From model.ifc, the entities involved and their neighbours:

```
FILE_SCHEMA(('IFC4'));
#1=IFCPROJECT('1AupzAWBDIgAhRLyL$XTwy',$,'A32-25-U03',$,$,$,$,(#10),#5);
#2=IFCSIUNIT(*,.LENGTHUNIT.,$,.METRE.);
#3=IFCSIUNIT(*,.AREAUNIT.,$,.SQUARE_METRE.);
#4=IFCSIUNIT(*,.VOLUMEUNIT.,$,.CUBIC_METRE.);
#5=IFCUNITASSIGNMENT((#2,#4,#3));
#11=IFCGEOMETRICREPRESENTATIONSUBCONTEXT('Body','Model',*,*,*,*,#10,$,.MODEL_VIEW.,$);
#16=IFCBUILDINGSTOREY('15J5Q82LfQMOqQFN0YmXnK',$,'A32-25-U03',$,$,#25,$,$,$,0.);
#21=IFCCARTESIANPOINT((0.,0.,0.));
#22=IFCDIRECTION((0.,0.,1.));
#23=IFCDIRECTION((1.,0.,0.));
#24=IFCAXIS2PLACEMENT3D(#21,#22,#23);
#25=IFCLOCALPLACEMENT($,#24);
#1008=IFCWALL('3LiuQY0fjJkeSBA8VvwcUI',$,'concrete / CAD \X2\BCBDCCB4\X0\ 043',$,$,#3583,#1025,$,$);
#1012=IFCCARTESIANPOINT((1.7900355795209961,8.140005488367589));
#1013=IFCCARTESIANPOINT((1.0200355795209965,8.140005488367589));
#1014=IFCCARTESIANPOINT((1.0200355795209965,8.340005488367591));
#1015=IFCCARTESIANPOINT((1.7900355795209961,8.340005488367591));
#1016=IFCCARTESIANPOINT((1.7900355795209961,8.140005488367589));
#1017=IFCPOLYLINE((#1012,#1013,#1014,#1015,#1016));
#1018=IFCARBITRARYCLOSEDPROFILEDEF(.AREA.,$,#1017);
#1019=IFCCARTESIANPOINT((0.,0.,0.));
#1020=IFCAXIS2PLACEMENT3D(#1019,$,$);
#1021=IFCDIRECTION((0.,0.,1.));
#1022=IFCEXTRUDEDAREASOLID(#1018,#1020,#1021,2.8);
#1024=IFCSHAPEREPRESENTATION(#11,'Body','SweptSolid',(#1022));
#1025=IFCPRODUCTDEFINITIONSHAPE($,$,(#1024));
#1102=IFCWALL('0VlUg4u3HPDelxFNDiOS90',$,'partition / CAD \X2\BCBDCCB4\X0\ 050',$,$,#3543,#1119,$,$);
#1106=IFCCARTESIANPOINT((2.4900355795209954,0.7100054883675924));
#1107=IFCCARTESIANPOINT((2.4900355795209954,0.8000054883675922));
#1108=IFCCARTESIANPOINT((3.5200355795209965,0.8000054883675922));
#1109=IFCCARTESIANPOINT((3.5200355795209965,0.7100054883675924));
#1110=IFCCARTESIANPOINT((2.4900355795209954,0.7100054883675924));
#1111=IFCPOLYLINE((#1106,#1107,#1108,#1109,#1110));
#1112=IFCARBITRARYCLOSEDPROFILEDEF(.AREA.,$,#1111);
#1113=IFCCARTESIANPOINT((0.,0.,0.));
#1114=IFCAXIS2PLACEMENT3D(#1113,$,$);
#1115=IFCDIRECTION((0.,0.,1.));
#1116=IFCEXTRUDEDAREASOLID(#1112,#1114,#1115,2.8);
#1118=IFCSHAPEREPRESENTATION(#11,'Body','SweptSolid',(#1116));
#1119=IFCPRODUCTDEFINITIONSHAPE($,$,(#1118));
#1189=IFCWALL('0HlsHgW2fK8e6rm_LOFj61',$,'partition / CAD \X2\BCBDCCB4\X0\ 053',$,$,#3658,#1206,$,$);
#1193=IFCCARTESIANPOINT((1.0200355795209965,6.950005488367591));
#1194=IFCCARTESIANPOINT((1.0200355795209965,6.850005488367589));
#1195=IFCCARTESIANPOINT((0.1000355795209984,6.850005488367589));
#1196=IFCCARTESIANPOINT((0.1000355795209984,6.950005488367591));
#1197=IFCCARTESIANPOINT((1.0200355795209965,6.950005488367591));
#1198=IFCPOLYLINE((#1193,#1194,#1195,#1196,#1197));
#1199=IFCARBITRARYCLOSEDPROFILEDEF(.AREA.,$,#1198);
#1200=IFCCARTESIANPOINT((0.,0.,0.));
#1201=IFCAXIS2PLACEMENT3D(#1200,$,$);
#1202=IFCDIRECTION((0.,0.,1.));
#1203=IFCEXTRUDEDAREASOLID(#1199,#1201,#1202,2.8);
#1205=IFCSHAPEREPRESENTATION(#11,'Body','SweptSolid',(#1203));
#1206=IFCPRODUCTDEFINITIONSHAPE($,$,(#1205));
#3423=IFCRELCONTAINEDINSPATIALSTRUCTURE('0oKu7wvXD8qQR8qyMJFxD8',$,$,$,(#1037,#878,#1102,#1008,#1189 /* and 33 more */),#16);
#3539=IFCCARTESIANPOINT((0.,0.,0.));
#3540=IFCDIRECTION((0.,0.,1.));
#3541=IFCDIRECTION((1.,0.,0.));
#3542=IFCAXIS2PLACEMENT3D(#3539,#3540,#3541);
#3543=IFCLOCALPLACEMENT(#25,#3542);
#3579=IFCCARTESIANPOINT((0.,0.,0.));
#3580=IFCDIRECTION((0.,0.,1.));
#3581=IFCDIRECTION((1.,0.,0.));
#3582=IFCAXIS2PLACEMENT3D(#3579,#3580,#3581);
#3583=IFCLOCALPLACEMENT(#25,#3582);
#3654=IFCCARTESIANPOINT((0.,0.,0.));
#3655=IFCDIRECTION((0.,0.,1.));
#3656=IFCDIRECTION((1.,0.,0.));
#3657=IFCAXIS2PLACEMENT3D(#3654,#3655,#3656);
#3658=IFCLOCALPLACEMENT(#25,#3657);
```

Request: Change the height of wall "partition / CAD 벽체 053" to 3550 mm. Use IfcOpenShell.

```python
import ifcopenshell
import ifcopenshell.geom
import ifcopenshell.util.representation
import ifcopenshell.util.shape

model = ifcopenshell.open("model.ifc")
settings = ifcopenshell.geom.settings()


def volume(element):
    """Net volume in cubic metres, openings subtracted."""
    shape = ifcopenshell.geom.create_shape(settings, element)
    return ifcopenshell.util.shape.get_volume(shape.geometry)


wall = model.by_id(1189)
before = volume(wall)

body = ifcopenshell.util.representation.get_representation(wall, "Model", "Body")
solid = body.Items[0]
old_height = solid.Depth
solid.Depth = 3.55
after = volume(wall)

print(f"height {old_height:g} -> {solid.Depth:g}, volume {before:.3f} -> {after:.3f} m3")

model.write("model_v2.ifc")
```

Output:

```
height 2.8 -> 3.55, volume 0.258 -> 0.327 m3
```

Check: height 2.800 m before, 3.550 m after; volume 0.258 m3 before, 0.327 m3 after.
